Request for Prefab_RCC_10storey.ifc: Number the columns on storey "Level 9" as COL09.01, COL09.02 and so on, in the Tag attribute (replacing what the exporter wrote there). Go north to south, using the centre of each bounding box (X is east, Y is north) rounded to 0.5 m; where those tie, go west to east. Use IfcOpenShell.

First a look at what the model holds.

```python
import ifcopenshell
import ifcopenshell.util.element
import ifcopenshell.util.placement

model = ifcopenshell.open("Prefab_RCC_10storey.ifc")
print(model.schema)
storey = next(s for s in model.by_type("IfcBuildingStorey") if s.Name == "Level 9")
columns = [e for e in ifcopenshell.util.element.get_decomposition(storey) if e.is_a("IfcColumn")]
for e in sorted(columns, key=lambda e: e.id()):
    origin = ifcopenshell.util.placement.get_local_placement(e.ObjectPlacement)[:3, 3]
    print(e.id(), e.Tag, e.Name, origin.round(2) + 0.0, sep=" | ")
```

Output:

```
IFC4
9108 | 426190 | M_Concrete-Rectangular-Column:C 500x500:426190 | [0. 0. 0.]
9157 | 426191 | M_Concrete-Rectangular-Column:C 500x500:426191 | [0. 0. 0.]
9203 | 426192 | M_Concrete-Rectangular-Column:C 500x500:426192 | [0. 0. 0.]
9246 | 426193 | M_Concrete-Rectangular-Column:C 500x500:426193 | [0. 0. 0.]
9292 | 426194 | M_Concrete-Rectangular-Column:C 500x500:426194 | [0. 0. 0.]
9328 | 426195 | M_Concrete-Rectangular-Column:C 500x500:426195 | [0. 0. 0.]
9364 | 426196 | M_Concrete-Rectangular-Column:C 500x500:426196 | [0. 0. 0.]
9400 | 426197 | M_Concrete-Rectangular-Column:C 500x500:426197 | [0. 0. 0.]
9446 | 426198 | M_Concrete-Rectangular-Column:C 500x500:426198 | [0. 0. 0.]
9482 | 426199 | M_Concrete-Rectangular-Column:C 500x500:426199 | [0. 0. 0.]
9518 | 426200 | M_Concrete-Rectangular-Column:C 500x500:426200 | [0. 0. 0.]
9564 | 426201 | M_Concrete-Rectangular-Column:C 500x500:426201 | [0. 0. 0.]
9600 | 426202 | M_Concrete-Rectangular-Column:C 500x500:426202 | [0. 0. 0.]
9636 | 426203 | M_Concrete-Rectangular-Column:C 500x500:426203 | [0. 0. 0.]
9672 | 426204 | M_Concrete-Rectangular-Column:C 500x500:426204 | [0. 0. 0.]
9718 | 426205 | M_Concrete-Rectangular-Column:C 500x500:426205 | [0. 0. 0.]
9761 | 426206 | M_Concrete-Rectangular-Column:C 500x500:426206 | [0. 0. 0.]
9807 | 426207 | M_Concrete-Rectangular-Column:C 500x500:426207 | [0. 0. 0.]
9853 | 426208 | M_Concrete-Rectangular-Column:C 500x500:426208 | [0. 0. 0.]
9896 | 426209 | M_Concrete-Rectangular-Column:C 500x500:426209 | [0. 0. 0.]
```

```python
import ifcopenshell
import ifcopenshell.geom
import ifcopenshell.util.element
import ifcopenshell.util.shape

model = ifcopenshell.open("Prefab_RCC_10storey.ifc")
settings = ifcopenshell.geom.settings()
settings.set("use-world-coords", True)


def centre(element):
    shape = ifcopenshell.geom.create_shape(settings, element)
    return ifcopenshell.util.shape.get_bbox_centroid(shape.geometry)


storey = next(s for s in model.by_type("IfcBuildingStorey") if s.Name == "Level 9")
columns = [e for e in ifcopenshell.util.element.get_decomposition(storey) if e.is_a("IfcColumn")]

# Insertion points can sit at a corner or the storey origin, so sort by the geometry (in metres).
centres = {e: centre(e) for e in columns}
columns.sort(key=lambda e: (-round(centres[e][1] / 0.5), centres[e][0]))

for i, e in enumerate(columns, start=1):
    number = f"COL09.{i:02d}"
    e.Tag = number
    print(e.id(), number)

model.write("Prefab_RCC_10storey-out.ifc")
```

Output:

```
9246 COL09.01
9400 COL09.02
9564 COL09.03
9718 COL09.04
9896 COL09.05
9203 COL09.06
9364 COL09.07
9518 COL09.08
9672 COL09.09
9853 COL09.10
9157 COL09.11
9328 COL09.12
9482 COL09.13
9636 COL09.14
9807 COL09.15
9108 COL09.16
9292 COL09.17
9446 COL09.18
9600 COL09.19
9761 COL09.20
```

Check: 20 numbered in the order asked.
